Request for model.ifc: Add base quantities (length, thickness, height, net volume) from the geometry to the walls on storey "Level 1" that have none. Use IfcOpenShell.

First a look at what the model holds.

```python
import ifcopenshell
import ifcopenshell.util.element
import ifcopenshell.util.unit

model = ifcopenshell.open("model.ifc")
print(model.schema)
for unit_type in ("LENGTHUNIT", "AREAUNIT", "VOLUMEUNIT"):
    print(unit_type, ifcopenshell.util.unit.calculate_unit_scale(model, unit_type))
storey = next(s for s in model.by_type("IfcBuildingStorey") if s.Name == "Level 1")
walls = [e for e in ifcopenshell.util.element.get_decomposition(storey) if e.is_a("IfcWall")]
for e in sorted(walls, key=lambda e: e.id()):
    print(e.id(), e.is_a(), e.Name, list(ifcopenshell.util.element.get_psets(e, qtos_only=True)), sep=" | ")
```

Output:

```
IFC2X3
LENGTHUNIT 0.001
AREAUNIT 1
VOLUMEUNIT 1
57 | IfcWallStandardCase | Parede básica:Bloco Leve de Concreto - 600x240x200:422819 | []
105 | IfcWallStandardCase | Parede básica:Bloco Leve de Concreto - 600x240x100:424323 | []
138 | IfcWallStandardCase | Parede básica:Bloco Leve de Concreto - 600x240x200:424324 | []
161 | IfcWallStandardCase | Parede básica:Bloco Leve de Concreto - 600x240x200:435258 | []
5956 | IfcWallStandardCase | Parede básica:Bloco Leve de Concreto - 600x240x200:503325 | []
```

```python
import ifcopenshell
import ifcopenshell.api.pset
import ifcopenshell.geom
import ifcopenshell.util.element
import ifcopenshell.util.shape
import ifcopenshell.util.unit

model = ifcopenshell.open("model.ifc")
unit_scale = ifcopenshell.util.unit.calculate_unit_scale(model)
volume_scale = ifcopenshell.util.unit.calculate_unit_scale(model, "VOLUMEUNIT")
settings = ifcopenshell.geom.settings()

storey = next(s for s in model.by_type("IfcBuildingStorey") if s.Name == "Level 1")
walls = [e for e in ifcopenshell.util.element.get_decomposition(storey) if e.is_a("IfcWall")]

for e in sorted(walls, key=lambda e: e.id()):
    if ifcopenshell.util.element.get_psets(e, qtos_only=True, should_inherit=False):
        continue
    # Geometry comes back in metres, in the element's own axes.
    shape = ifcopenshell.geom.create_shape(settings, e)
    values = {
        "Length": ifcopenshell.util.shape.get_x(shape.geometry) / unit_scale,
        "Width": ifcopenshell.util.shape.get_y(shape.geometry) / unit_scale,
        "Height": ifcopenshell.util.shape.get_z(shape.geometry) / unit_scale,
        "NetVolume": ifcopenshell.util.shape.get_volume(shape.geometry) / volume_scale,
    }
    qto = ifcopenshell.api.pset.add_qto(model, product=e, name="BaseQuantities")
    ifcopenshell.api.pset.edit_qto(model, qto=qto, properties=values)
    print(e.id(), {k: round(v, 3) for k, v in values.items()})

model.write("model_updated.ifc")
```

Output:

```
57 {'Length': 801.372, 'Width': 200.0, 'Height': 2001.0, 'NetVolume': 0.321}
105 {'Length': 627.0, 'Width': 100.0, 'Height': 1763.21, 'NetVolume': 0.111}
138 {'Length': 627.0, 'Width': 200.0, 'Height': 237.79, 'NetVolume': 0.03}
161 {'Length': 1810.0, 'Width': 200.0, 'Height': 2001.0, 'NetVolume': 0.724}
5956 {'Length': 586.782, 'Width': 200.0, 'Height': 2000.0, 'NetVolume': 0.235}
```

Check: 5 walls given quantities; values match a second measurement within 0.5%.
